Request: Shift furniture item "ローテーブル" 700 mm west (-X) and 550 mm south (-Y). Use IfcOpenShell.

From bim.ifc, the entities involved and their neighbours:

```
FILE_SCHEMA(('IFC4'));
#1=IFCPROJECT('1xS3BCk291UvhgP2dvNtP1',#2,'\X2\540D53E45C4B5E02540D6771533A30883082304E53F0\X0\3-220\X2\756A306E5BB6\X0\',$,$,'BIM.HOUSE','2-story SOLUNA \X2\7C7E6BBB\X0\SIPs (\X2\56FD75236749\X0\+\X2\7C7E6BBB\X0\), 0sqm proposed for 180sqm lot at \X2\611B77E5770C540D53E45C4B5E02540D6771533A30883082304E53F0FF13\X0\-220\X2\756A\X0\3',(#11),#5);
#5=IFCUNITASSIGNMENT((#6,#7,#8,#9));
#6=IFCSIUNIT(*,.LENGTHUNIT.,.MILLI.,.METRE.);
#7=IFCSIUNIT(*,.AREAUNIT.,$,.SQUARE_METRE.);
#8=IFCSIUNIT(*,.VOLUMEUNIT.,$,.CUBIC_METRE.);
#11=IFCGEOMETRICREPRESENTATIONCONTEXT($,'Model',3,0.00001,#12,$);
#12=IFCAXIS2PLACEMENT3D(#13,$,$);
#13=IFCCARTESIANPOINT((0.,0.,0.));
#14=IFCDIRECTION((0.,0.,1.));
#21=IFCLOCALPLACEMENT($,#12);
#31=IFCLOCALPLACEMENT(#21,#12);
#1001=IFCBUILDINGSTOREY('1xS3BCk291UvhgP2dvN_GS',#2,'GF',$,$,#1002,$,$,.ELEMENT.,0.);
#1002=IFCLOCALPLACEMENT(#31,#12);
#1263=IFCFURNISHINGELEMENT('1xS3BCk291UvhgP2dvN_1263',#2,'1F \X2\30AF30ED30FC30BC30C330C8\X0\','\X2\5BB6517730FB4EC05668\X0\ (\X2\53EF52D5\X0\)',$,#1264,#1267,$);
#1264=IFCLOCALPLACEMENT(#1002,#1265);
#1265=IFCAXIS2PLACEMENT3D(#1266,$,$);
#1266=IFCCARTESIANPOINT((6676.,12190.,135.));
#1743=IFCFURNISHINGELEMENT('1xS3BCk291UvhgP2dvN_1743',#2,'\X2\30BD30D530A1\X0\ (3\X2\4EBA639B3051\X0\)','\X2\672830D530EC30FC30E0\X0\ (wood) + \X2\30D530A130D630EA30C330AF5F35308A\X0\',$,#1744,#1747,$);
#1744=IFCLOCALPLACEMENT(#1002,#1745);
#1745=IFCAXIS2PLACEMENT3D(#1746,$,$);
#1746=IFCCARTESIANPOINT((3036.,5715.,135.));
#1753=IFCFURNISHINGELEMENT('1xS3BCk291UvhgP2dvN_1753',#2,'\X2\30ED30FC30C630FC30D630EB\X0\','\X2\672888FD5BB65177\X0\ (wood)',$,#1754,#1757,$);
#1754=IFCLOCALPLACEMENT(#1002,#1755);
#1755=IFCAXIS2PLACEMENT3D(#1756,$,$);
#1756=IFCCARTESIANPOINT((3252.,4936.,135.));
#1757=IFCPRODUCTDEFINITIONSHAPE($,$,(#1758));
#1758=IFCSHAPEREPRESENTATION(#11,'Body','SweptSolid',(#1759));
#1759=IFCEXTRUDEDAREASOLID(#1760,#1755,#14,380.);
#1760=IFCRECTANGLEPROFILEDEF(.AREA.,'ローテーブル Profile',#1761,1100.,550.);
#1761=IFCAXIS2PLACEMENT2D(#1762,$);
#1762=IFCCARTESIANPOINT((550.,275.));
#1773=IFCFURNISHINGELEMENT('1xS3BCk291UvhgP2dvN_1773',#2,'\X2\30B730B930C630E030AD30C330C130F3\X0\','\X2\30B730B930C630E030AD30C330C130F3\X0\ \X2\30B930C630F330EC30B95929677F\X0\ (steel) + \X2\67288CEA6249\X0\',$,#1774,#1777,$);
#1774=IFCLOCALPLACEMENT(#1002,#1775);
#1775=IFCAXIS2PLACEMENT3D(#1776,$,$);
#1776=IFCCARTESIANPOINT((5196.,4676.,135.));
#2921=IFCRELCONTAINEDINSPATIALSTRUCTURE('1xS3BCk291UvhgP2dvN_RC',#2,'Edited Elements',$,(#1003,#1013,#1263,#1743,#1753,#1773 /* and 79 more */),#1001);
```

```python
import ifcopenshell
import ifcopenshell.api.geometry
import ifcopenshell.util.placement
import ifcopenshell.util.unit

model = ifcopenshell.open("bim.ifc")
unit_scale = ifcopenshell.util.unit.calculate_unit_scale(model)

item = model.by_guid("1xS3BCk291UvhgP2dvN_1753")
matrix = ifcopenshell.util.placement.get_local_placement(item.ObjectPlacement)
matrix[0, 3] -= 0.7 / unit_scale
matrix[1, 3] -= 0.55 / unit_scale
ifcopenshell.api.geometry.edit_object_placement(model, product=item, matrix=matrix, is_si=False)

print(ifcopenshell.util.placement.get_local_placement(item.ObjectPlacement).round(3) + 0.0)

model.write("bim_v2.ifc")
```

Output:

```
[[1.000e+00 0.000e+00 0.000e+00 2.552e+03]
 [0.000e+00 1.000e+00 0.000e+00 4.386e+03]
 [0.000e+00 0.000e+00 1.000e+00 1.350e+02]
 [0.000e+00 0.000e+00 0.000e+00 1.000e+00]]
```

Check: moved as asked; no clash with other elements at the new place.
